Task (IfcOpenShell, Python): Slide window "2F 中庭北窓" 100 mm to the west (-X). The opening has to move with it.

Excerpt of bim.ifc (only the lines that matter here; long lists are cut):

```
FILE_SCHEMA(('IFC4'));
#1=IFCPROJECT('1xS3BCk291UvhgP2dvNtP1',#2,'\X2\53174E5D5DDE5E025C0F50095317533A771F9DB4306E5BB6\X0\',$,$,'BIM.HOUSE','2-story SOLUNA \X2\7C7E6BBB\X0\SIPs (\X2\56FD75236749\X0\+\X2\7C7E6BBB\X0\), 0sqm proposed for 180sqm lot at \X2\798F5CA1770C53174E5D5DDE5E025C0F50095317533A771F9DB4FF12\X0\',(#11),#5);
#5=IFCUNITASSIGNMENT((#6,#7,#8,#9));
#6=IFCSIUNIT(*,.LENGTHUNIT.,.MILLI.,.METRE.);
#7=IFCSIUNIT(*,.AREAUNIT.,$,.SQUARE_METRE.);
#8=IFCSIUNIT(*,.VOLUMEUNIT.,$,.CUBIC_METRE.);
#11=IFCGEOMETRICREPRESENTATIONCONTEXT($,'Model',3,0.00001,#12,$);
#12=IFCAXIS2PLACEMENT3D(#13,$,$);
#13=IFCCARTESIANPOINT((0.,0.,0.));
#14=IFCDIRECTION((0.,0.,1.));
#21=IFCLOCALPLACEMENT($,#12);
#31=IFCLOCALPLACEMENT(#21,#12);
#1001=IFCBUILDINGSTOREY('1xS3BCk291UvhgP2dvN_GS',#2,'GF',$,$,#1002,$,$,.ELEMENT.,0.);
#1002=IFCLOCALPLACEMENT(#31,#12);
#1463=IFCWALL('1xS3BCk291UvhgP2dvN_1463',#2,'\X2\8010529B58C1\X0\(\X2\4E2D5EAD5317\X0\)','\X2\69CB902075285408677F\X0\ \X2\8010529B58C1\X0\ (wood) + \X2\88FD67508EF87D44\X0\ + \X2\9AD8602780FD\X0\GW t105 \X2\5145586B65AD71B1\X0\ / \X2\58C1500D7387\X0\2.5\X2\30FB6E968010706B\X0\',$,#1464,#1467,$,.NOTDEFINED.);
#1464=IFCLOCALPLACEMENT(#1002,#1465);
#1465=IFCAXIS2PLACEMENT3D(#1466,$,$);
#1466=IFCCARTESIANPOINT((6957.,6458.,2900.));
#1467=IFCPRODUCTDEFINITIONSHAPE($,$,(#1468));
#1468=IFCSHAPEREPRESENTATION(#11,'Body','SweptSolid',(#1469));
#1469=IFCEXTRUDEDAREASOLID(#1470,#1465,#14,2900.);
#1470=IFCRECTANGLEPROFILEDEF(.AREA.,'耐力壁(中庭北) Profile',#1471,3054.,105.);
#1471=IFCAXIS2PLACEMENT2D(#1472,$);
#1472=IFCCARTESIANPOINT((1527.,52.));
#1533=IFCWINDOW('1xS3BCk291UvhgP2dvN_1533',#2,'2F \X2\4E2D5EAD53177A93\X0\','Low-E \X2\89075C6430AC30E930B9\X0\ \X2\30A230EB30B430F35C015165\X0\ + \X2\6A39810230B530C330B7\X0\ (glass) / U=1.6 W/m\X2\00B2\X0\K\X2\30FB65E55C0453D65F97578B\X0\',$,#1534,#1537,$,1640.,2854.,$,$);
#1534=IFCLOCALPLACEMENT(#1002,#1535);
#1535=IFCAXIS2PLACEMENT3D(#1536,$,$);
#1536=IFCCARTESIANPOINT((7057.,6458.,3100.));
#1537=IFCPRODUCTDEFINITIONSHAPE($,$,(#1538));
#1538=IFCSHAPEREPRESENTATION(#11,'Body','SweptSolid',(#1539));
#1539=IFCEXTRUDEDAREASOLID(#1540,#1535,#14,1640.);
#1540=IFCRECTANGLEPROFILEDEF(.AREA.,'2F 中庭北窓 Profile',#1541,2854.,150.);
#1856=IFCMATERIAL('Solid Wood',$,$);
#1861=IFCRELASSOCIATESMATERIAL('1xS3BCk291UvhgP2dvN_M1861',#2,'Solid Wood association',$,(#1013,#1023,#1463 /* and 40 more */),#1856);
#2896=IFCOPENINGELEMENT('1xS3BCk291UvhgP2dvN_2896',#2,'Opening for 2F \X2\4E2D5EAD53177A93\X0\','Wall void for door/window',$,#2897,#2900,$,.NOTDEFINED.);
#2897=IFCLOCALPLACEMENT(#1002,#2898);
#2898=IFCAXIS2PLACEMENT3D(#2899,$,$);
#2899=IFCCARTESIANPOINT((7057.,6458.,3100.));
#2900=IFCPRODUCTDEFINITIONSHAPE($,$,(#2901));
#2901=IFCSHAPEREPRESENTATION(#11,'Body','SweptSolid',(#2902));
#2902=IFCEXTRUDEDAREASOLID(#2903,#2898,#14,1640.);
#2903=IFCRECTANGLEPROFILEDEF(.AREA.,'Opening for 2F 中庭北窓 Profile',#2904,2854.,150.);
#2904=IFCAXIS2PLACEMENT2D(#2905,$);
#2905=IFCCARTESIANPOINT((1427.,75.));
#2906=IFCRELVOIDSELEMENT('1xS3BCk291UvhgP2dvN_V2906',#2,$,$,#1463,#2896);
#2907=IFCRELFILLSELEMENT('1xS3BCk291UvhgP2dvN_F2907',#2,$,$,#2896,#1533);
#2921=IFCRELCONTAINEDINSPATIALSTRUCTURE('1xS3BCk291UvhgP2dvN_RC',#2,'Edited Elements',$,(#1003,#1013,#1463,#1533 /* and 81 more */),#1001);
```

```python
import ifcopenshell
import ifcopenshell.api.geometry
import ifcopenshell.util.placement
import ifcopenshell.util.unit

model = ifcopenshell.open("bim.ifc")
unit_scale = ifcopenshell.util.unit.calculate_unit_scale(model)

window = model.by_id(1533)
opening = window.FillsVoids[0].RelatingOpeningElement
wall = opening.VoidsElements[0].RelatingBuildingElement

wall_matrix = ifcopenshell.util.placement.get_local_placement(wall.ObjectPlacement)
shift = wall_matrix[:3, 0] * -0.1 / unit_scale
before = ifcopenshell.util.placement.get_local_placement(window.ObjectPlacement)[:3, 3].copy()

# The window is not placed relative to its opening, so move both.
for product in (opening, window):
    matrix = ifcopenshell.util.placement.get_local_placement(product.ObjectPlacement)
    matrix[:3, 3] += shift
    ifcopenshell.api.geometry.edit_object_placement(model, product=product, matrix=matrix, is_si=False)

after = ifcopenshell.util.placement.get_local_placement(window.ObjectPlacement)[:3, 3]
print("window moved by", (after - before).round(3) + 0.0)

model.write("bim_rev.ifc")
```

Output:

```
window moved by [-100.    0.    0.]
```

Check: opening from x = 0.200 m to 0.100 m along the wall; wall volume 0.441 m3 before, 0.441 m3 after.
